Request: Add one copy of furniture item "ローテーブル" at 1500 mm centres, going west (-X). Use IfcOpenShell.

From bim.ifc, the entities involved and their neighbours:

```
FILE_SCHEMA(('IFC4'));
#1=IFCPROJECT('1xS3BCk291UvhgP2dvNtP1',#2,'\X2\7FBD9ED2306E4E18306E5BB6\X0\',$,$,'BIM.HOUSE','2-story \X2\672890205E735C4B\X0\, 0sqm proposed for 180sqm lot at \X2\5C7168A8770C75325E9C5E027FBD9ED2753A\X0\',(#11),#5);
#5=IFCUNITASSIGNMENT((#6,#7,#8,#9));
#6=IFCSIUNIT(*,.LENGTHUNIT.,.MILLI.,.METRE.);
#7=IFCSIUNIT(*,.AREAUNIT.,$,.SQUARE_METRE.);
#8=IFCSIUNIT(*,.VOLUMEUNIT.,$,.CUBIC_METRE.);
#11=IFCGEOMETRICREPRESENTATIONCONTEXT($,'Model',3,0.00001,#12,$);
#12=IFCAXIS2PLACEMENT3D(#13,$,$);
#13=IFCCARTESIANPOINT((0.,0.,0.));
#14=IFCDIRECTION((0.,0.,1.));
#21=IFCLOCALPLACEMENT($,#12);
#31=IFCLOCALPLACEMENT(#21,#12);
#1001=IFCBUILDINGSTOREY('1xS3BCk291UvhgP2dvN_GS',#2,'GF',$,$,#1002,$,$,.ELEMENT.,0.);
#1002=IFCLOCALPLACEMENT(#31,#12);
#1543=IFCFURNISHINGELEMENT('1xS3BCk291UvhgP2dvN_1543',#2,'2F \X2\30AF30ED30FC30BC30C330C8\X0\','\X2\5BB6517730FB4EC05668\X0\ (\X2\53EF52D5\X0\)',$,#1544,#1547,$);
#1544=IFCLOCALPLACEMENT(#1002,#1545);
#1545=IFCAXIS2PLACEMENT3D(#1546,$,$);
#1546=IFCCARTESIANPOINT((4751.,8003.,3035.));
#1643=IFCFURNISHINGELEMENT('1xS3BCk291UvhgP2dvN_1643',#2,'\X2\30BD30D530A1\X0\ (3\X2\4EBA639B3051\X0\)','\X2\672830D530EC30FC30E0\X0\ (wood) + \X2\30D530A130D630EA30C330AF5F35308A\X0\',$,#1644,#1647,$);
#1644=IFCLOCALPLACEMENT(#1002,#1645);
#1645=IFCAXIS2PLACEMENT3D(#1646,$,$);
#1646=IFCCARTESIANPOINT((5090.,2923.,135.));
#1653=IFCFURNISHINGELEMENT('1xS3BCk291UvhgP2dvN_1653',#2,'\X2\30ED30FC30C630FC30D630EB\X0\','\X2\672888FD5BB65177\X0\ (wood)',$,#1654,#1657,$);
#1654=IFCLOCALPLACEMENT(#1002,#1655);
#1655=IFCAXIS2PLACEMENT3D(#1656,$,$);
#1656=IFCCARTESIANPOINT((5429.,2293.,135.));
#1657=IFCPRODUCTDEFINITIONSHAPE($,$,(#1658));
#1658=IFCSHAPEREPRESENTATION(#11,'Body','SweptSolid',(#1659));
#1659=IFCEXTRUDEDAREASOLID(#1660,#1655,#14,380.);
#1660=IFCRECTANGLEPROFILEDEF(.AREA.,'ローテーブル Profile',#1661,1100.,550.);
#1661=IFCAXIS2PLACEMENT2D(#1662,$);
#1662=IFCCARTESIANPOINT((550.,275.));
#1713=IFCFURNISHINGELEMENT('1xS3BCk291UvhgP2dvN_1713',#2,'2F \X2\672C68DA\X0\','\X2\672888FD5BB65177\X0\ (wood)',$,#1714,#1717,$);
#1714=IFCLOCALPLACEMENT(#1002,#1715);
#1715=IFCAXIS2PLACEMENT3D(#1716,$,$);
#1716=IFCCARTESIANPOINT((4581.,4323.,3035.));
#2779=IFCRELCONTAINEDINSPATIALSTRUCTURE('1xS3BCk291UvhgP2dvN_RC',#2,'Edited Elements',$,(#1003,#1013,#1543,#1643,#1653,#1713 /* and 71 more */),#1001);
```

```python
import numpy as np
import ifcopenshell
import ifcopenshell.api.geometry
import ifcopenshell.api.root
import ifcopenshell.util.element
import ifcopenshell.util.placement

model = ifcopenshell.open("bim.ifc")


def reuse_history(source, copy):
    """copy_class also copies each property set's owner history, people and application; keep the originals."""
    for rel in copy.IsDefinedBy:
        if rel.is_a("IfcRelDefinesByProperties") and (history := rel.RelatingPropertyDefinition.OwnerHistory):
            rel.RelatingPropertyDefinition.OwnerHistory = source.OwnerHistory
            ifcopenshell.util.element.remove_deep2(model, history)


source = model.by_guid("1xS3BCk291UvhgP2dvN_1653")
base = ifcopenshell.util.placement.get_local_placement(source.ObjectPlacement)
step = np.array([-1.0, 0.0, 0.0]) * 1500.0

for i in range(1, 2):
    copy = ifcopenshell.api.root.copy_class(model, product=source)
    copy.Representation = ifcopenshell.util.element.copy_deep(
        model, source.Representation, exclude=["IfcGeometricRepresentationContext", "IfcRepresentationMap"]
    )
    reuse_history(source, copy)
    matrix = base.copy()
    matrix[:3, 3] += i * step
    print("added at", matrix[:3, 3].round(3) + 0.0)
    ifcopenshell.api.geometry.edit_object_placement(model, product=copy, matrix=matrix, is_si=False)

model.write("bim-out.ifc")
```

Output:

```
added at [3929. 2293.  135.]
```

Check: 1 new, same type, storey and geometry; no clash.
